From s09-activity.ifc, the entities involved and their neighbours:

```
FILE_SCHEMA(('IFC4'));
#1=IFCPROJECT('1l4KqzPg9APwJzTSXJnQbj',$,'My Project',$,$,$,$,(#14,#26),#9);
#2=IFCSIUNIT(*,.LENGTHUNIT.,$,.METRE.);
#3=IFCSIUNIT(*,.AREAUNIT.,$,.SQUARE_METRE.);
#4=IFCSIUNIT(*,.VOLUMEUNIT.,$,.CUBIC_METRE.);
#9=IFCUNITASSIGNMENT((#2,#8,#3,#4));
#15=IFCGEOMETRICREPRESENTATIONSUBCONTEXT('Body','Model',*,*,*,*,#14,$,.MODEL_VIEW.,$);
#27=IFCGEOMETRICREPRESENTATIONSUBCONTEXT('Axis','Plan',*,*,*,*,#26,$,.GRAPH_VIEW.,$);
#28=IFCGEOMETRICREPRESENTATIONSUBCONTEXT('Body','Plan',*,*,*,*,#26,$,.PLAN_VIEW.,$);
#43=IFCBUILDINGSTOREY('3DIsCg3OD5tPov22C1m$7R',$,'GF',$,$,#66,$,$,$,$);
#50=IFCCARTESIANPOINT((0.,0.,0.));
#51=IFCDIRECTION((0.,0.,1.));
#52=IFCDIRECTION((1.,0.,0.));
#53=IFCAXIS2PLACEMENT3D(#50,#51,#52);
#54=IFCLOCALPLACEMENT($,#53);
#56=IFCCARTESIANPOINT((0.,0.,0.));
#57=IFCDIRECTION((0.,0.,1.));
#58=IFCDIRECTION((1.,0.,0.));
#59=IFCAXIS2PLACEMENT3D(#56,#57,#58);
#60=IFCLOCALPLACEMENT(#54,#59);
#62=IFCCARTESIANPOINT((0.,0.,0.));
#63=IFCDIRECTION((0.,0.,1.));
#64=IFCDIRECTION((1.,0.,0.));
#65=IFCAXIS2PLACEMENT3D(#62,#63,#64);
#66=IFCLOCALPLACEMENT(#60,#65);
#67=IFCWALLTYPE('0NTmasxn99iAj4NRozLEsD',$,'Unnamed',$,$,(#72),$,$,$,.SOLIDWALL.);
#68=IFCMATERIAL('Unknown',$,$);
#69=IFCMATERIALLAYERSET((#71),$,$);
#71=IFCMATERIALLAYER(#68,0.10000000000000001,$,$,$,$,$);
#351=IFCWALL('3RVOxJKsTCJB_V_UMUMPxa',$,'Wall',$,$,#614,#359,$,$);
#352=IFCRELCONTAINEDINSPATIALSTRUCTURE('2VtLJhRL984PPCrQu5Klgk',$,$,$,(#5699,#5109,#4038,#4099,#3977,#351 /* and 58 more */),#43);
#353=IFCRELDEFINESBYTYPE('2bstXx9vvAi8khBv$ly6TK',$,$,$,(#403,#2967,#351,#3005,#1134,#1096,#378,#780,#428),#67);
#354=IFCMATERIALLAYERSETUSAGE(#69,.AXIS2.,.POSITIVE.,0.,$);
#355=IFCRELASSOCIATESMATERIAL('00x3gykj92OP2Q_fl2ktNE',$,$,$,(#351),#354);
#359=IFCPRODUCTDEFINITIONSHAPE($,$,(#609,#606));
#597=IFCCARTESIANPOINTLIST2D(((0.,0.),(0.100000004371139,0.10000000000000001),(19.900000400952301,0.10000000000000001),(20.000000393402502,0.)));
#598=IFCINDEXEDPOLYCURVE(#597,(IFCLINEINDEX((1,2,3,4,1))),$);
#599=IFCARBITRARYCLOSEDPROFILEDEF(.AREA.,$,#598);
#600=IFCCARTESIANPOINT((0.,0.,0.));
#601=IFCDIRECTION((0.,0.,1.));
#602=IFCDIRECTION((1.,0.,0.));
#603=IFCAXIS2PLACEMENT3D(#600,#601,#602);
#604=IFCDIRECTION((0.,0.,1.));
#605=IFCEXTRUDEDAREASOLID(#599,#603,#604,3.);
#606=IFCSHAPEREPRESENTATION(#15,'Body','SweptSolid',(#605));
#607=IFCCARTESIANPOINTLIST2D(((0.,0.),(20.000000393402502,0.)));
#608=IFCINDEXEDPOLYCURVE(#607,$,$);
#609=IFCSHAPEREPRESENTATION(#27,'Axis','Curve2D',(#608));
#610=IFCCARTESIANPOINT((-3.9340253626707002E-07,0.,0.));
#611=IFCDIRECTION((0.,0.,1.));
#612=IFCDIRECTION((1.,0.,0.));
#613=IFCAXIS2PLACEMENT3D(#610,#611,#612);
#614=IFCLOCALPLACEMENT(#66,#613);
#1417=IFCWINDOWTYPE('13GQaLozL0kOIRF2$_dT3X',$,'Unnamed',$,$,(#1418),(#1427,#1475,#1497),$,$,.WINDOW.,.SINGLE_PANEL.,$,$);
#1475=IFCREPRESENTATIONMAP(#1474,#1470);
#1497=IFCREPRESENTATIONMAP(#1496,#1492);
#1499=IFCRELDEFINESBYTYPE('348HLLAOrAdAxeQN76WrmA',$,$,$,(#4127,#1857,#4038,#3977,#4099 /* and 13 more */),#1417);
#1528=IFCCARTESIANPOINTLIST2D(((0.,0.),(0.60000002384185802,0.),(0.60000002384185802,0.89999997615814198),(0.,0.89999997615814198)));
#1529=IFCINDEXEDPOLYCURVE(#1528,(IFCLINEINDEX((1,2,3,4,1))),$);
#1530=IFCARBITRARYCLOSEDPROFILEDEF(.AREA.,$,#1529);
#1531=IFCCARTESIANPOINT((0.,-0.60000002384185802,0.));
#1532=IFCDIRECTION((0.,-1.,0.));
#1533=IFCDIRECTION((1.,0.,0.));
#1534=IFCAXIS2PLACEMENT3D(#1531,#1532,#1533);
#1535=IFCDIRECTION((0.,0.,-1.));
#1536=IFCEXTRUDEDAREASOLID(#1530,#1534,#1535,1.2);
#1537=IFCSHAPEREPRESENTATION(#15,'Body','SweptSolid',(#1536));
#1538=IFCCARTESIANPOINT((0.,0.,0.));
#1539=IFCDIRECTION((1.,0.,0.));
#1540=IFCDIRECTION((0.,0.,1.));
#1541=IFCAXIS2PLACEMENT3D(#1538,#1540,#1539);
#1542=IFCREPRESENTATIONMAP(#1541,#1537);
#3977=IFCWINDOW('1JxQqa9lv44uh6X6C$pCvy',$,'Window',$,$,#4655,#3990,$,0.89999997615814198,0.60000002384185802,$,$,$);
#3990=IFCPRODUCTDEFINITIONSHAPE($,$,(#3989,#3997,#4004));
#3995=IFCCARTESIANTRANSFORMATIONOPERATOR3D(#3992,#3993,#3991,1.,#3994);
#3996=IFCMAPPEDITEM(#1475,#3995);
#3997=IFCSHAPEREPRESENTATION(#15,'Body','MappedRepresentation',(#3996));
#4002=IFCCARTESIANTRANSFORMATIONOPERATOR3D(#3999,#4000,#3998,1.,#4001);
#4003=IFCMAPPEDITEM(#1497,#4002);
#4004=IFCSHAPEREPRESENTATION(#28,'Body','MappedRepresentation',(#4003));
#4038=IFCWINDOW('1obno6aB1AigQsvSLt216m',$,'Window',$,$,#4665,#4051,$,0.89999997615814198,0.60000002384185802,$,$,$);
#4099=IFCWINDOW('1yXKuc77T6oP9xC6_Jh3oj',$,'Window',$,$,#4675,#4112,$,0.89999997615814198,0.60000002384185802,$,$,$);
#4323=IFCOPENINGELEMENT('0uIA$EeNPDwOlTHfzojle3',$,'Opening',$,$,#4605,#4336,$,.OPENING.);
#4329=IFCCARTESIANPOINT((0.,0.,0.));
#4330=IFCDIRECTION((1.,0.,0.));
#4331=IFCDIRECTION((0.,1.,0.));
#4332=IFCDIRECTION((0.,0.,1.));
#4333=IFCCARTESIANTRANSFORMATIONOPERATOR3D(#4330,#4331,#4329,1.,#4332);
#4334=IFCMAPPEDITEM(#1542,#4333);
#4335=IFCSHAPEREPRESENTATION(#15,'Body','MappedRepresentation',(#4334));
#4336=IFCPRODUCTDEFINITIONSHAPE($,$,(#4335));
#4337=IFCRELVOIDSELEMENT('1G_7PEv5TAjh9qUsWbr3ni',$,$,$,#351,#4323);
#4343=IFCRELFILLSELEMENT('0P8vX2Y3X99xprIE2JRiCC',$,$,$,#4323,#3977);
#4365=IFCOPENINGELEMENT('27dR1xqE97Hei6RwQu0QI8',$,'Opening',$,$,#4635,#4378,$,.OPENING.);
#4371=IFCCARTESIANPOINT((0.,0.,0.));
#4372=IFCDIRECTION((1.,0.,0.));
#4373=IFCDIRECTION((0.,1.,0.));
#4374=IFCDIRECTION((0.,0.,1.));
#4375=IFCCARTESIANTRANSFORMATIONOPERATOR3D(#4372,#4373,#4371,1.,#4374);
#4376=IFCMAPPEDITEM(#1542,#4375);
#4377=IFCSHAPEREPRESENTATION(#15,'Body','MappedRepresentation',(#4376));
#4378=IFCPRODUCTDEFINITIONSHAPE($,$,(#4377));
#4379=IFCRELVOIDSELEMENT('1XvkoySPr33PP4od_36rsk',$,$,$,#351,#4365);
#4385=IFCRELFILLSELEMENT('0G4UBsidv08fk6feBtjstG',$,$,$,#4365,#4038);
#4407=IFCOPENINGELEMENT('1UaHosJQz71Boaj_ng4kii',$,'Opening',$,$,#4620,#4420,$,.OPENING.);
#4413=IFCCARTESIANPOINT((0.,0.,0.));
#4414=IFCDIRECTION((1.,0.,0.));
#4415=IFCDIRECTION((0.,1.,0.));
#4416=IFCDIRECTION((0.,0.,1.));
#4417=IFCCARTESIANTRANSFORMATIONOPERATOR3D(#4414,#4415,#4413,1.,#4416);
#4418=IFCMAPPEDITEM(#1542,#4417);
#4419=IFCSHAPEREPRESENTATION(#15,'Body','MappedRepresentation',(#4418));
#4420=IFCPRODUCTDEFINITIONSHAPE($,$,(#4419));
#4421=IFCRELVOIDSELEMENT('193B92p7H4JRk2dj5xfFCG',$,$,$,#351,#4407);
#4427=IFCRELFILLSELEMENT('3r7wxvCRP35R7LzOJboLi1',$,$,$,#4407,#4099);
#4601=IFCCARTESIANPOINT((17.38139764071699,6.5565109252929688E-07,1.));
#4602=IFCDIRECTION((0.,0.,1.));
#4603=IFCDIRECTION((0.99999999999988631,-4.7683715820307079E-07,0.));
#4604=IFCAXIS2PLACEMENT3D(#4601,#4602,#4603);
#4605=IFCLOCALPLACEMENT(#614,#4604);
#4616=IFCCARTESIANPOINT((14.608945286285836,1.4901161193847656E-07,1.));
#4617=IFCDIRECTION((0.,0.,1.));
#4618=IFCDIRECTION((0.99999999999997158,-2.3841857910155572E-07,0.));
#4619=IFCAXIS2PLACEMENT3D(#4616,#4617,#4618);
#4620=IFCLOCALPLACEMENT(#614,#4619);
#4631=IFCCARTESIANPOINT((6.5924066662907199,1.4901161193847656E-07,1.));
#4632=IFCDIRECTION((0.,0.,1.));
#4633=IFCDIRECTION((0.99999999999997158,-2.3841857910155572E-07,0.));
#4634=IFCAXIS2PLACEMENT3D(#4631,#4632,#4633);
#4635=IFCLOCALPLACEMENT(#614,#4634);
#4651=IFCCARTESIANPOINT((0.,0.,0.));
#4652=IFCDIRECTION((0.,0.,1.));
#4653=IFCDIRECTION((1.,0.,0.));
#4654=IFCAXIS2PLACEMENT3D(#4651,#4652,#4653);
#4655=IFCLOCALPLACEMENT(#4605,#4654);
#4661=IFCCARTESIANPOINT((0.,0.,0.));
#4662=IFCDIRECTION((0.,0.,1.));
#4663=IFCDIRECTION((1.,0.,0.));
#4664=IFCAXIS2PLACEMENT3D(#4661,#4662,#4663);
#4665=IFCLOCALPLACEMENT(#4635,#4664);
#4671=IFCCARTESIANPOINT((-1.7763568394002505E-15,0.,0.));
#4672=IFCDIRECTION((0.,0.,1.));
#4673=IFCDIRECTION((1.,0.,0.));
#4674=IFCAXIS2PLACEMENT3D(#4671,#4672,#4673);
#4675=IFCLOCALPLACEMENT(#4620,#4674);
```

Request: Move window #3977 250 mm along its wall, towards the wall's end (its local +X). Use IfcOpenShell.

```python
import ifcopenshell
import ifcopenshell.api.geometry
import ifcopenshell.util.placement
import ifcopenshell.util.unit

model = ifcopenshell.open("s09-activity.ifc")
unit_scale = ifcopenshell.util.unit.calculate_unit_scale(model)

window = model.by_guid("1JxQqa9lv44uh6X6C$pCvy")
opening = window.FillsVoids[0].RelatingOpeningElement
wall = opening.VoidsElements[0].RelatingBuildingElement

wall_matrix = ifcopenshell.util.placement.get_local_placement(wall.ObjectPlacement)
shift = wall_matrix[:3, 0] * 0.25 / unit_scale
before = ifcopenshell.util.placement.get_local_placement(window.ObjectPlacement)[:3, 3].copy()

# The window is placed relative to its opening, so it follows when the opening moves.
matrix = ifcopenshell.util.placement.get_local_placement(opening.ObjectPlacement)
matrix[:3, 3] += shift
ifcopenshell.api.geometry.edit_object_placement(
    model, product=opening, matrix=matrix, is_si=False, should_transform_children=True
)

after = ifcopenshell.util.placement.get_local_placement(window.ObjectPlacement)[:3, 3]
print("window moved by", (after - before).round(3) + 0.0)

model.write("s09-activity_v2.ifc")
```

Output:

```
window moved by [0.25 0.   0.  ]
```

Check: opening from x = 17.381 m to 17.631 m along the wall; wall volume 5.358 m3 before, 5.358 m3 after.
